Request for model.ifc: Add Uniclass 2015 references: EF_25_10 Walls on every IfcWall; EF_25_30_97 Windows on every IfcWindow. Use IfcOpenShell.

First a look at what the model holds.

```python
import ifcopenshell

model = ifcopenshell.open("model.ifc")
print(model.schema)
print("classifications:", [c.Name for c in model.by_type("IfcClassification")])
for ifc_class in ("IfcDoor", "IfcRoof", "IfcStair", "IfcWall", "IfcWindow"):
    print(ifc_class, len(model.by_type(ifc_class)))
```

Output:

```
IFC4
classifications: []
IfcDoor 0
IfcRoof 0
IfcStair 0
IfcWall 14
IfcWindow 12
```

```python
import ifcopenshell
import ifcopenshell.api.classification

model = ifcopenshell.open("model.ifc")

system = ifcopenshell.api.classification.add_classification(model, classification="Uniclass 2015")

codes = {
    "IfcWall": ("EF_25_10", "Walls"),
    "IfcWindow": ("EF_25_30_97", "Windows"),
}
for ifc_class, (code, name) in codes.items():
    products = model.by_type(ifc_class)
    ifcopenshell.api.classification.add_reference(
        model, products=products, classification=system, identification=code, name=name
    )
    print(code, len(products))

model.write("model_updated.ifc")
```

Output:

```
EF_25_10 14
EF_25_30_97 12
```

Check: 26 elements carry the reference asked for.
